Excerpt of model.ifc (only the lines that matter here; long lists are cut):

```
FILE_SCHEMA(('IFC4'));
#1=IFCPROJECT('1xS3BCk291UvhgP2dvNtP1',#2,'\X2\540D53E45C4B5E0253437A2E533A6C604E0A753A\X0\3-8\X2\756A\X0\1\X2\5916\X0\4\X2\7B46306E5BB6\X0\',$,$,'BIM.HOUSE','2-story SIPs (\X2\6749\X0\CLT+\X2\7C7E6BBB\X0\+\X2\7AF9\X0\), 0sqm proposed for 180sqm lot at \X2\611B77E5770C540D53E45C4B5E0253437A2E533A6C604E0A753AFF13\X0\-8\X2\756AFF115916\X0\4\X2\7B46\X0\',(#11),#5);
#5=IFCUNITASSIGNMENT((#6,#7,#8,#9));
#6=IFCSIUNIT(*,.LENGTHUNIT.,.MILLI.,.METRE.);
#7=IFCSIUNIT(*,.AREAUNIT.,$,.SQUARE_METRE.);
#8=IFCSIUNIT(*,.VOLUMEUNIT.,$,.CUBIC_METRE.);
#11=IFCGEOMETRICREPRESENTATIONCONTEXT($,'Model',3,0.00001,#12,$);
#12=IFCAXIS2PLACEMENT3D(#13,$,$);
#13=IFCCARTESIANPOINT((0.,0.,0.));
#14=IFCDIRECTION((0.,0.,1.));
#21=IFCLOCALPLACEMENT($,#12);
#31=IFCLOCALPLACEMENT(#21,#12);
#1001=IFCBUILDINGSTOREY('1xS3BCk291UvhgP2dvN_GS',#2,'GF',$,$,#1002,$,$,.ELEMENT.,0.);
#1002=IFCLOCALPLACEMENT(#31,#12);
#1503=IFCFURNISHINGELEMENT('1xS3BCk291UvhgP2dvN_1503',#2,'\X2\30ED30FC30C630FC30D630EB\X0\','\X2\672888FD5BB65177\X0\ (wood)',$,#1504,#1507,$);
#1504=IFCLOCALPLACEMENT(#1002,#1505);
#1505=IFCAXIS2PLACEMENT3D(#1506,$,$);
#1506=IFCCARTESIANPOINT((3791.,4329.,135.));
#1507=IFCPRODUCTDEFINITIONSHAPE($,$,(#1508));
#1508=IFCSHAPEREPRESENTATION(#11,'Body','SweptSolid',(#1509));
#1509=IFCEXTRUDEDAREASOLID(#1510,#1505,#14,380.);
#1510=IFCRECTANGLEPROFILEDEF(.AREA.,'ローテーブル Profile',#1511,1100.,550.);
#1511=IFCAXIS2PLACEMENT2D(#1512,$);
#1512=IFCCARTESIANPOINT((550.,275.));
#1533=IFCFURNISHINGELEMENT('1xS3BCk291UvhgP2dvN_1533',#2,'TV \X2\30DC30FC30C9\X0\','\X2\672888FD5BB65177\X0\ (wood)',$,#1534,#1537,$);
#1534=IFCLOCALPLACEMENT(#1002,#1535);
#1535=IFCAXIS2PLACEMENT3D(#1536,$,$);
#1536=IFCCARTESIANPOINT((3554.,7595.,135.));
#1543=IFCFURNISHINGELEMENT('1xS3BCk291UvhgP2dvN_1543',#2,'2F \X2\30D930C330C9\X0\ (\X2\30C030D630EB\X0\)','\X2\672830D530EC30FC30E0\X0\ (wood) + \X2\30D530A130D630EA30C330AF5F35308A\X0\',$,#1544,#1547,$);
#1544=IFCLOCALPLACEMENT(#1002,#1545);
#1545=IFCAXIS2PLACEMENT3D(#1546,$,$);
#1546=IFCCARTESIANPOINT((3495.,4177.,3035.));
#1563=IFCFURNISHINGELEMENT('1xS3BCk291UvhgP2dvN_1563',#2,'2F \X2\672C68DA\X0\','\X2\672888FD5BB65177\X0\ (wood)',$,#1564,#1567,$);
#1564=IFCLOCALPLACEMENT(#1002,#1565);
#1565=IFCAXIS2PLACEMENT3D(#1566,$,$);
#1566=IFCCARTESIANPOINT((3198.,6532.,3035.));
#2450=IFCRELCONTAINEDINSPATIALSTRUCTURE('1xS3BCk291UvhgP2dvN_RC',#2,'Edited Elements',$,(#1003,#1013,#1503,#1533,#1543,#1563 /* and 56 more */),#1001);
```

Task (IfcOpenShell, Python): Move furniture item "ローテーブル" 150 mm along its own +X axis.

```python
import ifcopenshell
import ifcopenshell.api.geometry
import ifcopenshell.util.placement
import ifcopenshell.util.unit

model = ifcopenshell.open("model.ifc")
unit_scale = ifcopenshell.util.unit.calculate_unit_scale(model)

item = model.by_guid("1xS3BCk291UvhgP2dvN_1503")
matrix = ifcopenshell.util.placement.get_local_placement(item.ObjectPlacement)
matrix[:3, 3] += matrix[:3, 0] * 0.15 / unit_scale
ifcopenshell.api.geometry.edit_object_placement(model, product=item, matrix=matrix, is_si=False)

print(ifcopenshell.util.placement.get_local_placement(item.ObjectPlacement).round(3) + 0.0)

model.write("model_rev.ifc")
```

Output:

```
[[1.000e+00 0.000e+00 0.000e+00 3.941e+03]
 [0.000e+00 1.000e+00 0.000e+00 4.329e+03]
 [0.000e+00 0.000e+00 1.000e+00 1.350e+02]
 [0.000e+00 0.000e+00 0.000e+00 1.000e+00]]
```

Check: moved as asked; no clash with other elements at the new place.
